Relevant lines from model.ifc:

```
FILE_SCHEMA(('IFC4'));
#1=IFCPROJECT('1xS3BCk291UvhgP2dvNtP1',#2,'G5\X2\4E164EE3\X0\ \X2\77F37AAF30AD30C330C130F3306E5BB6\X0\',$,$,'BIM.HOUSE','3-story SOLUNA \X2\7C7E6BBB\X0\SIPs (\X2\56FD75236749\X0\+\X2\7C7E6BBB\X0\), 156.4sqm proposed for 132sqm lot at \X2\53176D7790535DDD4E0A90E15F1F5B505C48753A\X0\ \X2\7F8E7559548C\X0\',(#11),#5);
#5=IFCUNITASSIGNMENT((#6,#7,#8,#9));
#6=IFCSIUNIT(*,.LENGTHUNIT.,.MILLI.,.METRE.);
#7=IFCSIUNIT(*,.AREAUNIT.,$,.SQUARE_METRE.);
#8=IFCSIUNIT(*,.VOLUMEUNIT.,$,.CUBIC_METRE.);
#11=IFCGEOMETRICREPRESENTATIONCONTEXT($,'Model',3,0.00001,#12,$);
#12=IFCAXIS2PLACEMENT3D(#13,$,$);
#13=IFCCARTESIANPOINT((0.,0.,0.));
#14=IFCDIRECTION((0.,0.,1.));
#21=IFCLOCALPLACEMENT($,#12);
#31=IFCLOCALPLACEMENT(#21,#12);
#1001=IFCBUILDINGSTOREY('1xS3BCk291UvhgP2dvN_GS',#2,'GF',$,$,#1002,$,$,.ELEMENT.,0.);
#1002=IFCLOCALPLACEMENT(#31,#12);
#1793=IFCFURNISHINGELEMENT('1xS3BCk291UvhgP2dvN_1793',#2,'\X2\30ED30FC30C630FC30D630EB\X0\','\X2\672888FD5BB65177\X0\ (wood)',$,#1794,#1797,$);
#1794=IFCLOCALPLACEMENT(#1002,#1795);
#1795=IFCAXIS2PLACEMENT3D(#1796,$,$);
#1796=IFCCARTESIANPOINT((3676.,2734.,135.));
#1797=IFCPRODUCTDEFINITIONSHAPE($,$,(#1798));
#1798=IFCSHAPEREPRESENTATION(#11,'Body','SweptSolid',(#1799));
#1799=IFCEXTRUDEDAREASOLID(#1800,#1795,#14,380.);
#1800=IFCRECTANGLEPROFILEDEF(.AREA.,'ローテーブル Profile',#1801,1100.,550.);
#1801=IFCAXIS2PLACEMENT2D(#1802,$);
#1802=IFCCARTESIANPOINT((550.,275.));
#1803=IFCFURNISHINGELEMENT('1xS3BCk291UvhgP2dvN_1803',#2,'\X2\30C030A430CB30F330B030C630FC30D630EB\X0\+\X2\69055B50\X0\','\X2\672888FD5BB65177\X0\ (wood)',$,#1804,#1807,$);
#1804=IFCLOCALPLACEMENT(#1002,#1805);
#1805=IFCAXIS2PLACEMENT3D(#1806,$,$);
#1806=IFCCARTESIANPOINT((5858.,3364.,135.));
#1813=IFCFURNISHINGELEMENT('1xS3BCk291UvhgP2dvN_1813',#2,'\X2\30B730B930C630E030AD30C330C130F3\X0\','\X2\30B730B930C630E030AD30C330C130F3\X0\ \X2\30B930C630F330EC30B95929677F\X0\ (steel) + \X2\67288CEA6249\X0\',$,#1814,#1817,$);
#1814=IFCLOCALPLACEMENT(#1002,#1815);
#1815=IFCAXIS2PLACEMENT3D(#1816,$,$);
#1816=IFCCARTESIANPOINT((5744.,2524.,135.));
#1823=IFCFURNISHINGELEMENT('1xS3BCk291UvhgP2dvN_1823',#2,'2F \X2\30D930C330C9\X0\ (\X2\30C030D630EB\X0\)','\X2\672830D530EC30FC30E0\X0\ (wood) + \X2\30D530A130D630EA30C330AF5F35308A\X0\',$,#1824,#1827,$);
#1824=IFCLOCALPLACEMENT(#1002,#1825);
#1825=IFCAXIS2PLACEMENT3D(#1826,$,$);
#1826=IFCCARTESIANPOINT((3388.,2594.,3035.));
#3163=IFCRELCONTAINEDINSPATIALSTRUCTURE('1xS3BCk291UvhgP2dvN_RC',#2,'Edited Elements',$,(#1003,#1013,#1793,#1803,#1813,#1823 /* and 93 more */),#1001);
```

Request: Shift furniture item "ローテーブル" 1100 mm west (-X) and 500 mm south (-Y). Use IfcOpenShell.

```python
import ifcopenshell
import ifcopenshell.api.geometry
import ifcopenshell.util.placement
import ifcopenshell.util.unit

model = ifcopenshell.open("model.ifc")
unit_scale = ifcopenshell.util.unit.calculate_unit_scale(model)

item = model.by_id(1793)
matrix = ifcopenshell.util.placement.get_local_placement(item.ObjectPlacement)
matrix[0, 3] -= 1.1 / unit_scale
matrix[1, 3] -= 0.5 / unit_scale
ifcopenshell.api.geometry.edit_object_placement(model, product=item, matrix=matrix, is_si=False)

print(ifcopenshell.util.placement.get_local_placement(item.ObjectPlacement).round(3) + 0.0)

model.write("model-out.ifc")
```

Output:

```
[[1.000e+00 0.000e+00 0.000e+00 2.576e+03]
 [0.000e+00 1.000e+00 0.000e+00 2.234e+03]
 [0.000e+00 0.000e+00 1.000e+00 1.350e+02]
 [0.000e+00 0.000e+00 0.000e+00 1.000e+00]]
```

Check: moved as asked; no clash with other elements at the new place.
